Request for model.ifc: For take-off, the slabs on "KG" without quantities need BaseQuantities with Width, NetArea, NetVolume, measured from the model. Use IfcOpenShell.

First a look at what the model holds.

```python
import ifcopenshell
import ifcopenshell.util.element
import ifcopenshell.util.unit

model = ifcopenshell.open("model.ifc")
print(model.schema)
for unit_type in ("LENGTHUNIT", "AREAUNIT", "VOLUMEUNIT"):
    print(unit_type, ifcopenshell.util.unit.calculate_unit_scale(model, unit_type))
storey = next(s for s in model.by_type("IfcBuildingStorey") if s.Name == "KG")
slabs = [e for e in ifcopenshell.util.element.get_decomposition(storey) if e.is_a("IfcSlab")]
for e in sorted(slabs, key=lambda e: e.id()):
    print(e.id(), e.is_a(), e.Name, list(ifcopenshell.util.element.get_psets(e, qtos_only=True)), sep=" | ")
```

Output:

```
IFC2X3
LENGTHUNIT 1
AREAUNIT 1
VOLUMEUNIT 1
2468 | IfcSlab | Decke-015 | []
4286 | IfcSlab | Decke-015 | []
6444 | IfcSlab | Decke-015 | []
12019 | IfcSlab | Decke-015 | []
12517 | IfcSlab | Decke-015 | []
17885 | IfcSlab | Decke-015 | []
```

```python
import ifcopenshell
import ifcopenshell.api.pset
import ifcopenshell.geom
import ifcopenshell.util.element
import ifcopenshell.util.shape
import ifcopenshell.util.unit

model = ifcopenshell.open("model.ifc")
unit_scale = ifcopenshell.util.unit.calculate_unit_scale(model)
area_scale = ifcopenshell.util.unit.calculate_unit_scale(model, "AREAUNIT")
volume_scale = ifcopenshell.util.unit.calculate_unit_scale(model, "VOLUMEUNIT")
settings = ifcopenshell.geom.settings()

storey = next(s for s in model.by_type("IfcBuildingStorey") if s.Name == "KG")
slabs = [e for e in ifcopenshell.util.element.get_decomposition(storey) if e.is_a("IfcSlab")]

for e in sorted(slabs, key=lambda e: e.id()):
    if ifcopenshell.util.element.get_psets(e, qtos_only=True, should_inherit=False):
        continue
    # Geometry comes back in metres, in the element's own axes.
    shape = ifcopenshell.geom.create_shape(settings, e)
    values = {
        "Width": ifcopenshell.util.shape.get_z(shape.geometry) / unit_scale,
        "NetArea": ifcopenshell.util.shape.get_footprint_area(shape.geometry) / area_scale,
        "NetVolume": ifcopenshell.util.shape.get_volume(shape.geometry) / volume_scale,
    }
    qto = ifcopenshell.api.pset.add_qto(model, product=e, name="BaseQuantities")
    ifcopenshell.api.pset.edit_qto(model, qto=qto, properties=values)
    print(e.id(), {k: round(v, 3) for k, v in values.items()})

model.write("model_edited.ifc")
```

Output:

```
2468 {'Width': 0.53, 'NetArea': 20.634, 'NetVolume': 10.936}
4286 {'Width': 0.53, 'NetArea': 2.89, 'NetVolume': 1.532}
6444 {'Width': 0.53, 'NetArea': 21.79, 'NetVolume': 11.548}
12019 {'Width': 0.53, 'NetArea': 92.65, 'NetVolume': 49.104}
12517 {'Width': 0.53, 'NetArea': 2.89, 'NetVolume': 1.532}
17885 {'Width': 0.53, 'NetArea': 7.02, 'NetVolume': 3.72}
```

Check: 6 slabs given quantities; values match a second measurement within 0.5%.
